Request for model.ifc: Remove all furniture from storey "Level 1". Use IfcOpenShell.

First a look at what the model holds.

```python
import ifcopenshell
import ifcopenshell.util.element

model = ifcopenshell.open("model.ifc")
print(model.schema)
storey = next(s for s in model.by_type("IfcBuildingStorey") if s.Name == "Level 1")
furniture = [e for e in ifcopenshell.util.element.get_decomposition(storey) if e.is_a("IfcFurnishingElement")]
seen = {}
for e in furniture:
    element_type = ifcopenshell.util.element.get_type(e)
    name = element_type.Name if element_type not in (None, e) else None
    seen[name] = seen.get(name, 0) + 1
for name, count in sorted(seen.items(), key=str):
    print(count, "x", name)
```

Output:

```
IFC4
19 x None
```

```python
import ifcopenshell
import ifcopenshell.api.root
import ifcopenshell.util.element

model = ifcopenshell.open("model.ifc")

storey = next(s for s in model.by_type("IfcBuildingStorey") if s.Name == "Level 1")
furniture = [e for e in ifcopenshell.util.element.get_decomposition(storey) if e.is_a("IfcFurnishingElement")]

for e in furniture:
    ifcopenshell.api.root.remove_product(model, product=e)
print(len(furniture), "removed")

model.write("model_v2.ifc")
```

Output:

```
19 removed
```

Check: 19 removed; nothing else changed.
